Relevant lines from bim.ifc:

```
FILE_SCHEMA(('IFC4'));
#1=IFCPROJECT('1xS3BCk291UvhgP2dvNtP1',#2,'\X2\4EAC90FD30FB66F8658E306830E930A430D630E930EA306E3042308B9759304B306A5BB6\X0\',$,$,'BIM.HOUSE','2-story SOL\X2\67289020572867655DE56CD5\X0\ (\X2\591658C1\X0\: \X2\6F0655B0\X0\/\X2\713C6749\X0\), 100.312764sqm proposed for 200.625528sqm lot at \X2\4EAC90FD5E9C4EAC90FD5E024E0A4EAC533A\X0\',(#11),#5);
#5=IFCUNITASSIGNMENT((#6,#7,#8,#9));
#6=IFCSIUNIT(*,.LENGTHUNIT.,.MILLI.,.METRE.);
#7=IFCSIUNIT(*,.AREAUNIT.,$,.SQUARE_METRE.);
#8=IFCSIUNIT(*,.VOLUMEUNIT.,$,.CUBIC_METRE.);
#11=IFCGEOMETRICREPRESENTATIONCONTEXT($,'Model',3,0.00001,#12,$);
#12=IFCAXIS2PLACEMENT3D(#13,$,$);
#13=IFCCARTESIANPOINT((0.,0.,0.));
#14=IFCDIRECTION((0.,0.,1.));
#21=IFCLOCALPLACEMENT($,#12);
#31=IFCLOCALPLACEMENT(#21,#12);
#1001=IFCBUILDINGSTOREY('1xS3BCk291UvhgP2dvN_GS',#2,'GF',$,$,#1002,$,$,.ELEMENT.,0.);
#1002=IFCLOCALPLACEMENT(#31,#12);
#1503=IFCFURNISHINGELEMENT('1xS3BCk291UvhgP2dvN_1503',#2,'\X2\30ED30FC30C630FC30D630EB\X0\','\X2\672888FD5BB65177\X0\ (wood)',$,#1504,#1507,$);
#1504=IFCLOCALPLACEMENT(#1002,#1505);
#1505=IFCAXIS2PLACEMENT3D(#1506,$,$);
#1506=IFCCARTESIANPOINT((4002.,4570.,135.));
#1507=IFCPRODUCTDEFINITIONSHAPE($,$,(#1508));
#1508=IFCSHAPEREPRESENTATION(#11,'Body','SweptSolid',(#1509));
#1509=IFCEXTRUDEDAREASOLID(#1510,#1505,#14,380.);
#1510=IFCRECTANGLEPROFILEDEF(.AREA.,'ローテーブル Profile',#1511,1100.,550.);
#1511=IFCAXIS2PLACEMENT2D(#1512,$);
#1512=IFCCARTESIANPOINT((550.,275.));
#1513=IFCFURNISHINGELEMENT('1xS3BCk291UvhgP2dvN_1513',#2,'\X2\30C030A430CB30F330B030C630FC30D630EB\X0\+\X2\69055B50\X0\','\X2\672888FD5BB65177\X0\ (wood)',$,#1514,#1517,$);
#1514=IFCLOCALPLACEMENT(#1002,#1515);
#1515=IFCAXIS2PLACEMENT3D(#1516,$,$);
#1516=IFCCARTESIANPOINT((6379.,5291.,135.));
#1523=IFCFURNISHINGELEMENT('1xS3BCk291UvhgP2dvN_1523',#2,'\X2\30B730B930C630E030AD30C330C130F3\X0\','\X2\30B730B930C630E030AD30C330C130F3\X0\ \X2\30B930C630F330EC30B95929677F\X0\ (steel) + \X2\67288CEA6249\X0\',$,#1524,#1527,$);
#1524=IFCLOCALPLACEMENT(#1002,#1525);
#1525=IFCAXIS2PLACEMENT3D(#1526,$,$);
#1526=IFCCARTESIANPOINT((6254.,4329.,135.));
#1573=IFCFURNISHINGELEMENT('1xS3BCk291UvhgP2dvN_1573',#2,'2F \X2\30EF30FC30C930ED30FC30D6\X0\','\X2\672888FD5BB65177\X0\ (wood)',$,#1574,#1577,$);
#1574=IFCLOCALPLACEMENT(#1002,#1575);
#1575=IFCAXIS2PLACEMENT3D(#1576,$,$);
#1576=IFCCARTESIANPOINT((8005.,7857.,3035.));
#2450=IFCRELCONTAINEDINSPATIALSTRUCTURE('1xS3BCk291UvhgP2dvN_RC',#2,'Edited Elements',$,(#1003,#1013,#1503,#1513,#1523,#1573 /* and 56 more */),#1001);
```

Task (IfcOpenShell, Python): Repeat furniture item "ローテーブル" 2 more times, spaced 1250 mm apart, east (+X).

```python
import numpy as np
import ifcopenshell
import ifcopenshell.api.geometry
import ifcopenshell.api.root
import ifcopenshell.util.element
import ifcopenshell.util.placement

model = ifcopenshell.open("bim.ifc")


def reuse_history(source, copy):
    """copy_class also copies each property set's owner history, people and application; keep the originals."""
    for rel in copy.IsDefinedBy:
        if rel.is_a("IfcRelDefinesByProperties") and (history := rel.RelatingPropertyDefinition.OwnerHistory):
            rel.RelatingPropertyDefinition.OwnerHistory = source.OwnerHistory
            ifcopenshell.util.element.remove_deep2(model, history)


source = model.by_id(1503)
base = ifcopenshell.util.placement.get_local_placement(source.ObjectPlacement)
step = np.array([1.0, 0.0, 0.0]) * 1250.0

for i in range(1, 3):
    copy = ifcopenshell.api.root.copy_class(model, product=source)
    copy.Representation = ifcopenshell.util.element.copy_deep(
        model, source.Representation, exclude=["IfcGeometricRepresentationContext", "IfcRepresentationMap"]
    )
    reuse_history(source, copy)
    matrix = base.copy()
    matrix[:3, 3] += i * step
    print("added at", matrix[:3, 3].round(3) + 0.0)
    ifcopenshell.api.geometry.edit_object_placement(model, product=copy, matrix=matrix, is_si=False)

model.write("bim_rev.ifc")
```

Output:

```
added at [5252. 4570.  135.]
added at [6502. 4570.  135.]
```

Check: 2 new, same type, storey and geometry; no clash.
